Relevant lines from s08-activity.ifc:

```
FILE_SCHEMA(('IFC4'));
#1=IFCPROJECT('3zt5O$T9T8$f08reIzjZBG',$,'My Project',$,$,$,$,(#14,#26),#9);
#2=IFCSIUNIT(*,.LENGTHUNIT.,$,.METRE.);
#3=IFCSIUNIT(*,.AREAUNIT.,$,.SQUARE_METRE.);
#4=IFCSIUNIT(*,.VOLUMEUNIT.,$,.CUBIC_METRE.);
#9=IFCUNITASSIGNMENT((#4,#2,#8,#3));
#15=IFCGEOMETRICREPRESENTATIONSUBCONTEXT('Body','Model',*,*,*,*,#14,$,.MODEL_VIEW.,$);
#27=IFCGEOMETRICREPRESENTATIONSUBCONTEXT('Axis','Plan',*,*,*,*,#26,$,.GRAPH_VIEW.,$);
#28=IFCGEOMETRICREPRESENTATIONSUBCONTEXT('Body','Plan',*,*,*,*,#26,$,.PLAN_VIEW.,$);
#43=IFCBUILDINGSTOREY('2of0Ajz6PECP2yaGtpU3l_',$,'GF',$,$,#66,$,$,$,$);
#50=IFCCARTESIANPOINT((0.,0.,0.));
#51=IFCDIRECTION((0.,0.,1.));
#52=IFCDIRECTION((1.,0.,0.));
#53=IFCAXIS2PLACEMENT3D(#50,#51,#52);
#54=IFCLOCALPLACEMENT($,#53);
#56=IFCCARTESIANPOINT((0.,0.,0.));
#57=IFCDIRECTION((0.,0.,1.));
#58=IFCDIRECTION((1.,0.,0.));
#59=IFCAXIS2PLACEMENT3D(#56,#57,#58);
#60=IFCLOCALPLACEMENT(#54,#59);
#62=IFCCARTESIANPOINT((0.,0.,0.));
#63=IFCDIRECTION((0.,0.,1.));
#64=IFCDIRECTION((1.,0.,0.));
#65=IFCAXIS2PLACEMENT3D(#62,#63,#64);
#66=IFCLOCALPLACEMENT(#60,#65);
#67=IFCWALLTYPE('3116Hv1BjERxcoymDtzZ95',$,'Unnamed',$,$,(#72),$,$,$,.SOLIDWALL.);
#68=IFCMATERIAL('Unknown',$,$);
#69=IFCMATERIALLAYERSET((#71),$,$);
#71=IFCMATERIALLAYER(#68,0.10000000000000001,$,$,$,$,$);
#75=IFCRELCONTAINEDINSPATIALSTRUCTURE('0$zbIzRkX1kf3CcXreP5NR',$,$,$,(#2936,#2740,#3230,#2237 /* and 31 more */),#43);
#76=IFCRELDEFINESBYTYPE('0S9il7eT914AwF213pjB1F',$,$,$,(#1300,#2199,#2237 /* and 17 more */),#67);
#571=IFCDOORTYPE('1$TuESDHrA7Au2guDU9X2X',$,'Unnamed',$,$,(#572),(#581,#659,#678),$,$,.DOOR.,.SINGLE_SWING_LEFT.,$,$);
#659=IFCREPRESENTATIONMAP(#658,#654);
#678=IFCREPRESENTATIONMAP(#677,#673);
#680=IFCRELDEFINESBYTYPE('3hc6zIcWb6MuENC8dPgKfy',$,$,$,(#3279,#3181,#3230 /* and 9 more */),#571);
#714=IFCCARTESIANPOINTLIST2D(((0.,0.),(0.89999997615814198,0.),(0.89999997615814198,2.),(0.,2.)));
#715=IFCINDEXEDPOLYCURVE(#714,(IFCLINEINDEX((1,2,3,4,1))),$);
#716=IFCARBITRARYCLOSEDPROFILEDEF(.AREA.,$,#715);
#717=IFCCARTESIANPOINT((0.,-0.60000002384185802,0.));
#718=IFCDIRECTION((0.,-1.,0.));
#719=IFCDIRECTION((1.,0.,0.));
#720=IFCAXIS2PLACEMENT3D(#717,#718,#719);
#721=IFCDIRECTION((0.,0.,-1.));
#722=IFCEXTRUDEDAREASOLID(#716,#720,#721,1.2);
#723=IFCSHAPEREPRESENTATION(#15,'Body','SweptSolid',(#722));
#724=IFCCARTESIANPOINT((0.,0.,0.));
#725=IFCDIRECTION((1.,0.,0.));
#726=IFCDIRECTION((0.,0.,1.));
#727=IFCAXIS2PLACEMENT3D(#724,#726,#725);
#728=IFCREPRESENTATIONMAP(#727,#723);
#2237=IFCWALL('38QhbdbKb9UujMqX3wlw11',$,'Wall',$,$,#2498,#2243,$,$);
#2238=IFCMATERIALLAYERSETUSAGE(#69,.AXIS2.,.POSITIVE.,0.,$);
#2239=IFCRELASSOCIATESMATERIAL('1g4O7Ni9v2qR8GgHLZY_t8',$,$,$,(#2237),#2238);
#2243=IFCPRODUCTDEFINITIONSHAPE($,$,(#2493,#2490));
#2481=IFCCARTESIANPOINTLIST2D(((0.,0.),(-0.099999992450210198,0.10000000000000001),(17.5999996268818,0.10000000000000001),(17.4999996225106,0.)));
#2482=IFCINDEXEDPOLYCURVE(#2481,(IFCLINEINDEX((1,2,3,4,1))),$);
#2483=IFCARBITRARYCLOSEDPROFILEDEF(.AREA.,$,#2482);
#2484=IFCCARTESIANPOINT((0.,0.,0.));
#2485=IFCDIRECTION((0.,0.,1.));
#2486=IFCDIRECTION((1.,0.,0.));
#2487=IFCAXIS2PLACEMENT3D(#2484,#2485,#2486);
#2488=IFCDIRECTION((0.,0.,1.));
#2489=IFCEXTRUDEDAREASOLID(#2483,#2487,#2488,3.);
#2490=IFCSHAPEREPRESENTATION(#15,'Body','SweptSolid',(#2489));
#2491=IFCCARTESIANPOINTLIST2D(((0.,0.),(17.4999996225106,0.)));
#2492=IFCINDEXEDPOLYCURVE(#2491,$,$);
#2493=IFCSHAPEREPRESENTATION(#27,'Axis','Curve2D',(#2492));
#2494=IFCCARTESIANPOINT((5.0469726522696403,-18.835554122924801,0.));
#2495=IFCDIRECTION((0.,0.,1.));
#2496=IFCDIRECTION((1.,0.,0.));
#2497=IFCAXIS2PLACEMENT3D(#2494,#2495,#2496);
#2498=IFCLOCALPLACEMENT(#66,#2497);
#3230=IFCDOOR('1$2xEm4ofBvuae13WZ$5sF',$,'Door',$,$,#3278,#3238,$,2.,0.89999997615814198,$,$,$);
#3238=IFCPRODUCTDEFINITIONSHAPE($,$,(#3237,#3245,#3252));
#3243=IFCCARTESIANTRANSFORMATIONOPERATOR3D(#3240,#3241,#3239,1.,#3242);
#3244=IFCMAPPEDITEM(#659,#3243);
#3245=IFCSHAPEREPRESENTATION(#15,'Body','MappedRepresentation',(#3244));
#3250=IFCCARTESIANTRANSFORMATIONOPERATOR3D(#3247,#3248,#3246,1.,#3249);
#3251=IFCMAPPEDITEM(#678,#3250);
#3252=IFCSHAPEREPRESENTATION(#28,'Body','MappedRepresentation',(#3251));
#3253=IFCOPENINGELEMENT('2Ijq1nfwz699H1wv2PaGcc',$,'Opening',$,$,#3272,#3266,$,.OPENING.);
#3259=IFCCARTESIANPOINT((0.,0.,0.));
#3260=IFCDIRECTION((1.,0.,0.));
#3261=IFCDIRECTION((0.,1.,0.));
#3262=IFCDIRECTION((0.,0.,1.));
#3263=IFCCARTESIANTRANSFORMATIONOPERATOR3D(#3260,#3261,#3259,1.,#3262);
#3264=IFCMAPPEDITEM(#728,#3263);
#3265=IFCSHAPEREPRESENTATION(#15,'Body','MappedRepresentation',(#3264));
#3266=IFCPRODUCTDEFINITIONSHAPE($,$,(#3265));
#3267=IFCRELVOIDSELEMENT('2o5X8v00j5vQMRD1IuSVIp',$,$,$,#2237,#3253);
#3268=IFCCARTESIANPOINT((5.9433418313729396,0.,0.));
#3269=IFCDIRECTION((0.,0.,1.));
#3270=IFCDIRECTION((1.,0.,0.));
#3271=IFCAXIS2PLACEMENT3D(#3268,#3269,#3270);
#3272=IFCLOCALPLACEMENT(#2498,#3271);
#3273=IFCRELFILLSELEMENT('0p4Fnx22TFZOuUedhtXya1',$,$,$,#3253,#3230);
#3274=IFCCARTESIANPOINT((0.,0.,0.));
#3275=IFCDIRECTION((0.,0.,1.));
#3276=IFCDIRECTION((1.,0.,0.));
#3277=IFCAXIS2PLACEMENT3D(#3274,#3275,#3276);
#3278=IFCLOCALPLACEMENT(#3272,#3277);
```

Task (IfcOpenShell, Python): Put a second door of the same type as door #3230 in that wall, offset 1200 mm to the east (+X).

```python
import ifcopenshell
import ifcopenshell.api.feature
import ifcopenshell.api.geometry
import ifcopenshell.api.root
import ifcopenshell.geom
import ifcopenshell.util.element
import ifcopenshell.util.placement
import ifcopenshell.util.shape
import ifcopenshell.util.unit

model = ifcopenshell.open("s08-activity.ifc")
unit_scale = ifcopenshell.util.unit.calculate_unit_scale(model)
settings = ifcopenshell.geom.settings()


def volume(element):
    """Net volume in cubic metres, openings subtracted."""
    shape = ifcopenshell.geom.create_shape(settings, element)
    return ifcopenshell.util.shape.get_volume(shape.geometry)


door = model.by_guid("1$2xEm4ofBvuae13WZ$5sF")
opening = door.FillsVoids[0].RelatingOpeningElement
wall = opening.VoidsElements[0].RelatingBuildingElement
before = volume(wall)
shift = ifcopenshell.util.placement.get_local_placement(wall.ObjectPlacement)[:3, 0] * 1.2 / unit_scale

# copy_class copies the void relationship, type, container and properties, but no geometry.
new_opening = ifcopenshell.api.root.copy_class(model, product=opening)
new_opening.Representation = ifcopenshell.util.element.copy_deep(
    model, opening.Representation, exclude=["IfcGeometricRepresentationContext", "IfcRepresentationMap"]
)
new_door = ifcopenshell.api.root.copy_class(model, product=door)
new_door.Representation = ifcopenshell.util.element.copy_deep(
    model, door.Representation, exclude=["IfcGeometricRepresentationContext", "IfcRepresentationMap"]
)
ifcopenshell.api.feature.add_filling(model, opening=new_opening, element=new_door)

for old, new in ((opening, new_opening), (door, new_door)):
    matrix = ifcopenshell.util.placement.get_local_placement(old.ObjectPlacement)
    matrix[:3, 3] += shift
    ifcopenshell.api.geometry.edit_object_placement(model, product=new, matrix=matrix, is_si=False)

after = volume(wall)

print(f"wall volume {before:.3f} -> {after:.3f} m3")

model.write("s08-activity_edited.ifc")
```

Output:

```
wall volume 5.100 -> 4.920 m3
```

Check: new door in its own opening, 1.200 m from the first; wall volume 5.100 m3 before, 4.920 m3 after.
